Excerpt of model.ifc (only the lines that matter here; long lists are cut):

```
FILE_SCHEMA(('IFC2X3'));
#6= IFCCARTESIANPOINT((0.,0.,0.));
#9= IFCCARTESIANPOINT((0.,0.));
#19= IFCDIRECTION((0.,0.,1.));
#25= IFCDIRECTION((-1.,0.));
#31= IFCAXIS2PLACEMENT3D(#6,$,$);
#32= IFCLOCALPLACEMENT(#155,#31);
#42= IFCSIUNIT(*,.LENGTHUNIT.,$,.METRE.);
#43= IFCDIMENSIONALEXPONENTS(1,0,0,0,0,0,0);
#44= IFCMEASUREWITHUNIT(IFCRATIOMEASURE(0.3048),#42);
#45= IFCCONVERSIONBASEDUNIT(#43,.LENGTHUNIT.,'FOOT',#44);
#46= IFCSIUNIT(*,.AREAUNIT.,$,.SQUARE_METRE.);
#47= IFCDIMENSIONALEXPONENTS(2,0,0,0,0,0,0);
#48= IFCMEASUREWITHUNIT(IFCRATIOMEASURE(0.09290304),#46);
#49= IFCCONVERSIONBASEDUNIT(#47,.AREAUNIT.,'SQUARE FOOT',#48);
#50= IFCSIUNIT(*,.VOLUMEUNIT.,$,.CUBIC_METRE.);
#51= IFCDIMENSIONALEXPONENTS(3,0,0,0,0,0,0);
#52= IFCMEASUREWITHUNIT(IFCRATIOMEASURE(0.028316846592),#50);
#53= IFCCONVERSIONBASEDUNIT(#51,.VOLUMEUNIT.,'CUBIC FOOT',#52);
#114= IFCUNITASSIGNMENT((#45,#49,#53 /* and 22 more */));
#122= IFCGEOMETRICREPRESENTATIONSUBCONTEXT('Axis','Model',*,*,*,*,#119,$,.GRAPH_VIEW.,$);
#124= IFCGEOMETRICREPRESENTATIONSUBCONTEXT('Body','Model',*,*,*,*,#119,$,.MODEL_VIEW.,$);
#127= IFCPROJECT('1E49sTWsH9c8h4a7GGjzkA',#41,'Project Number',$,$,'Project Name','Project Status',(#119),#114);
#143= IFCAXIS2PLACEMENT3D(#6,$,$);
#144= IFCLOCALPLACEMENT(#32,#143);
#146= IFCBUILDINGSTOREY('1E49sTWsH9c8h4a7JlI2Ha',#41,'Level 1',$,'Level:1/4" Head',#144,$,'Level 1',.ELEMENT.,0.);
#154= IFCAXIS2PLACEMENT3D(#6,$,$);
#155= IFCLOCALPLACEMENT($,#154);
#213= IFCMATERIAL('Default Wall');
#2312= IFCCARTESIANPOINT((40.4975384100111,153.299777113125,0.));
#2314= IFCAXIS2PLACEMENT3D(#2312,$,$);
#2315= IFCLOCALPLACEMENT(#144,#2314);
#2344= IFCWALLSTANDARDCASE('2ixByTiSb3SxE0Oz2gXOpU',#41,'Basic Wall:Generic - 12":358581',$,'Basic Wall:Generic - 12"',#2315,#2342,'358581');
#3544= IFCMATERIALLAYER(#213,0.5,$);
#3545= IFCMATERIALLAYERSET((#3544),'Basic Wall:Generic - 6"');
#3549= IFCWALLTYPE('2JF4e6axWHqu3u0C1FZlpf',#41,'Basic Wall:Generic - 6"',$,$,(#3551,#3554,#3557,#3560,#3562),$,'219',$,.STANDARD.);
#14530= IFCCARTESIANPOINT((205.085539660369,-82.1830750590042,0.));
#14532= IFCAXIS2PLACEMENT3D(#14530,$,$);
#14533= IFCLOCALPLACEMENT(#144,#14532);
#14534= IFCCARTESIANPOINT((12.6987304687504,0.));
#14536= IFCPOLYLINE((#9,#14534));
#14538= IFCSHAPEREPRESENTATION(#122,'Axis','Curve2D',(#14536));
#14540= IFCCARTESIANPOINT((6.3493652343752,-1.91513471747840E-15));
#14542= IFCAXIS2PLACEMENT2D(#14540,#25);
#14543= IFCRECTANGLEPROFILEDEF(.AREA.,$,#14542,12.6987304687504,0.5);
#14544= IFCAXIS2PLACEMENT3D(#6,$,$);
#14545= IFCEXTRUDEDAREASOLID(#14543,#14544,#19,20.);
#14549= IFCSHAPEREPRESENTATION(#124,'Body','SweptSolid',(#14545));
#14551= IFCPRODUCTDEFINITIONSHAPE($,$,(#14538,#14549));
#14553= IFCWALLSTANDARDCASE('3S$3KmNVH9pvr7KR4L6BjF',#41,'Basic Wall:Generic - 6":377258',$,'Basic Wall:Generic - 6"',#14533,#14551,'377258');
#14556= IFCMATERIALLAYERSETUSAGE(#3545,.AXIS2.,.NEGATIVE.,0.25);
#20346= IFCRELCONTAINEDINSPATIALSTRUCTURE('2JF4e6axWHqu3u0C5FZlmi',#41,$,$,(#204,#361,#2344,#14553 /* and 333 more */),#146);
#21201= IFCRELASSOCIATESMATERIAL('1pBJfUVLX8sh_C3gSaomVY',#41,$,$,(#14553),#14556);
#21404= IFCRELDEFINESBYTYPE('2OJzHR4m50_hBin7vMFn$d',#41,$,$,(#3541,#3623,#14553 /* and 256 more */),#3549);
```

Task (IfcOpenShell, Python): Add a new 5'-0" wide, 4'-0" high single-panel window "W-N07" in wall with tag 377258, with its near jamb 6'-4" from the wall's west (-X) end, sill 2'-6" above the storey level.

```python
import numpy as np
import ifcopenshell
import ifcopenshell.api.feature
import ifcopenshell.api.geometry
import ifcopenshell.api.root
import ifcopenshell.api.spatial
import ifcopenshell.api.type
import ifcopenshell.geom
import ifcopenshell.util.element
import ifcopenshell.util.placement
import ifcopenshell.util.representation
import ifcopenshell.util.shape
import ifcopenshell.util.unit

model = ifcopenshell.open("model.ifc")
unit_scale = ifcopenshell.util.unit.calculate_unit_scale(model)
settings = ifcopenshell.geom.settings()


def volume(element):
    """Net volume in cubic metres, openings subtracted."""
    shape = ifcopenshell.geom.create_shape(settings, element)
    return ifcopenshell.util.shape.get_volume(shape.geometry)


wall = model.by_id(14553)
storey = ifcopenshell.util.element.get_container(wall, ifc_class="IfcBuildingStorey")
context = ifcopenshell.util.representation.get_context(model, "Model", "Body", "MODEL_VIEW")
before = volume(wall)

width, height, from_end, sill = 1.524, 1.2192, 1.9304, 0.762  # metres

# The wall runs along its own X axis, and the end named is its -X end.
wall_shape = ifcopenshell.geom.create_shape(settings, wall)
x, y, z = ifcopenshell.util.shape.get_vertices(wall_shape.geometry).T
start = x.min() + from_end
face, thickness = float(y.min()), float(y.max() - y.min())
wall_matrix = ifcopenshell.util.placement.get_local_placement(wall.ObjectPlacement)
level = ifcopenshell.util.placement.get_local_placement(storey.ObjectPlacement)[2, 3]


def in_wall(x, y):
    """Placement at x, y metres in the wall's axes, at sill height."""
    matrix = wall_matrix.copy()
    matrix[:, 3] = wall_matrix @ np.array([x / unit_scale, y / unit_scale, 0.0, 1.0])
    matrix[2, 3] = level + sill / unit_scale
    return matrix


# Opening: a box that overshoots both wall faces by 50 mm.
opening = ifcopenshell.api.root.create_entity(model, ifc_class="IfcOpeningElement")
box = ifcopenshell.api.geometry.add_wall_representation(
    model, context=context, length=width, height=height, thickness=thickness + 0.1
)
ifcopenshell.api.geometry.assign_representation(model, product=opening, representation=box)
ifcopenshell.api.geometry.edit_object_placement(model, product=opening, matrix=in_wall(start, face - 0.05), is_si=False)
ifcopenshell.api.feature.add_feature(model, feature=opening, element=wall)

window = ifcopenshell.api.root.create_entity(model, ifc_class="IfcWindow", name="W-N07")
window.OverallWidth, window.OverallHeight = width / unit_scale, height / unit_scale
body = ifcopenshell.api.geometry.add_window_representation(
    model,
    context=context,
    overall_width=window.OverallWidth,
    overall_height=window.OverallHeight,
    partition_type="SINGLE_PANEL",
)
ifcopenshell.api.geometry.assign_representation(model, product=window, representation=body)
ifcopenshell.api.spatial.assign_container(model, products=[window], relating_structure=storey)
fills = ifcopenshell.api.feature.add_filling(model, opening=opening, element=window)
fills.OwnerHistory = window.OwnerHistory  # required in IFC2X3

# IFC2X3 keeps the operation on the window style.
style = ifcopenshell.api.root.create_entity(model, ifc_class="IfcWindowStyle", name="W-N07")
style.OperationType, style.ConstructionType = "SINGLE_PANEL", "NOTDEFINED"
style.ParameterTakesPrecedence = style.Sizeable = False
ifcopenshell.api.type.assign_type(model, related_objects=[window], relating_type=style)

# Centre the window in the wall's thickness.
ifcopenshell.api.geometry.edit_object_placement(model, product=window, matrix=in_wall(start, face), is_si=False)
window_shape = ifcopenshell.geom.create_shape(settings, window)
depth = ifcopenshell.util.shape.get_vertices(window_shape.geometry)[:, 1]
offset = face + thickness / 2 - (depth.min() + depth.max()) / 2
ifcopenshell.api.geometry.edit_object_placement(model, product=window, matrix=in_wall(start, offset), is_si=False)

after = volume(wall)

print(f"wall volume {before:.3f} -> {after:.3f} m3")

model.write("model_edited.ifc")
```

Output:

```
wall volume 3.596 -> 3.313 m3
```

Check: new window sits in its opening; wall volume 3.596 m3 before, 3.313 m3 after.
